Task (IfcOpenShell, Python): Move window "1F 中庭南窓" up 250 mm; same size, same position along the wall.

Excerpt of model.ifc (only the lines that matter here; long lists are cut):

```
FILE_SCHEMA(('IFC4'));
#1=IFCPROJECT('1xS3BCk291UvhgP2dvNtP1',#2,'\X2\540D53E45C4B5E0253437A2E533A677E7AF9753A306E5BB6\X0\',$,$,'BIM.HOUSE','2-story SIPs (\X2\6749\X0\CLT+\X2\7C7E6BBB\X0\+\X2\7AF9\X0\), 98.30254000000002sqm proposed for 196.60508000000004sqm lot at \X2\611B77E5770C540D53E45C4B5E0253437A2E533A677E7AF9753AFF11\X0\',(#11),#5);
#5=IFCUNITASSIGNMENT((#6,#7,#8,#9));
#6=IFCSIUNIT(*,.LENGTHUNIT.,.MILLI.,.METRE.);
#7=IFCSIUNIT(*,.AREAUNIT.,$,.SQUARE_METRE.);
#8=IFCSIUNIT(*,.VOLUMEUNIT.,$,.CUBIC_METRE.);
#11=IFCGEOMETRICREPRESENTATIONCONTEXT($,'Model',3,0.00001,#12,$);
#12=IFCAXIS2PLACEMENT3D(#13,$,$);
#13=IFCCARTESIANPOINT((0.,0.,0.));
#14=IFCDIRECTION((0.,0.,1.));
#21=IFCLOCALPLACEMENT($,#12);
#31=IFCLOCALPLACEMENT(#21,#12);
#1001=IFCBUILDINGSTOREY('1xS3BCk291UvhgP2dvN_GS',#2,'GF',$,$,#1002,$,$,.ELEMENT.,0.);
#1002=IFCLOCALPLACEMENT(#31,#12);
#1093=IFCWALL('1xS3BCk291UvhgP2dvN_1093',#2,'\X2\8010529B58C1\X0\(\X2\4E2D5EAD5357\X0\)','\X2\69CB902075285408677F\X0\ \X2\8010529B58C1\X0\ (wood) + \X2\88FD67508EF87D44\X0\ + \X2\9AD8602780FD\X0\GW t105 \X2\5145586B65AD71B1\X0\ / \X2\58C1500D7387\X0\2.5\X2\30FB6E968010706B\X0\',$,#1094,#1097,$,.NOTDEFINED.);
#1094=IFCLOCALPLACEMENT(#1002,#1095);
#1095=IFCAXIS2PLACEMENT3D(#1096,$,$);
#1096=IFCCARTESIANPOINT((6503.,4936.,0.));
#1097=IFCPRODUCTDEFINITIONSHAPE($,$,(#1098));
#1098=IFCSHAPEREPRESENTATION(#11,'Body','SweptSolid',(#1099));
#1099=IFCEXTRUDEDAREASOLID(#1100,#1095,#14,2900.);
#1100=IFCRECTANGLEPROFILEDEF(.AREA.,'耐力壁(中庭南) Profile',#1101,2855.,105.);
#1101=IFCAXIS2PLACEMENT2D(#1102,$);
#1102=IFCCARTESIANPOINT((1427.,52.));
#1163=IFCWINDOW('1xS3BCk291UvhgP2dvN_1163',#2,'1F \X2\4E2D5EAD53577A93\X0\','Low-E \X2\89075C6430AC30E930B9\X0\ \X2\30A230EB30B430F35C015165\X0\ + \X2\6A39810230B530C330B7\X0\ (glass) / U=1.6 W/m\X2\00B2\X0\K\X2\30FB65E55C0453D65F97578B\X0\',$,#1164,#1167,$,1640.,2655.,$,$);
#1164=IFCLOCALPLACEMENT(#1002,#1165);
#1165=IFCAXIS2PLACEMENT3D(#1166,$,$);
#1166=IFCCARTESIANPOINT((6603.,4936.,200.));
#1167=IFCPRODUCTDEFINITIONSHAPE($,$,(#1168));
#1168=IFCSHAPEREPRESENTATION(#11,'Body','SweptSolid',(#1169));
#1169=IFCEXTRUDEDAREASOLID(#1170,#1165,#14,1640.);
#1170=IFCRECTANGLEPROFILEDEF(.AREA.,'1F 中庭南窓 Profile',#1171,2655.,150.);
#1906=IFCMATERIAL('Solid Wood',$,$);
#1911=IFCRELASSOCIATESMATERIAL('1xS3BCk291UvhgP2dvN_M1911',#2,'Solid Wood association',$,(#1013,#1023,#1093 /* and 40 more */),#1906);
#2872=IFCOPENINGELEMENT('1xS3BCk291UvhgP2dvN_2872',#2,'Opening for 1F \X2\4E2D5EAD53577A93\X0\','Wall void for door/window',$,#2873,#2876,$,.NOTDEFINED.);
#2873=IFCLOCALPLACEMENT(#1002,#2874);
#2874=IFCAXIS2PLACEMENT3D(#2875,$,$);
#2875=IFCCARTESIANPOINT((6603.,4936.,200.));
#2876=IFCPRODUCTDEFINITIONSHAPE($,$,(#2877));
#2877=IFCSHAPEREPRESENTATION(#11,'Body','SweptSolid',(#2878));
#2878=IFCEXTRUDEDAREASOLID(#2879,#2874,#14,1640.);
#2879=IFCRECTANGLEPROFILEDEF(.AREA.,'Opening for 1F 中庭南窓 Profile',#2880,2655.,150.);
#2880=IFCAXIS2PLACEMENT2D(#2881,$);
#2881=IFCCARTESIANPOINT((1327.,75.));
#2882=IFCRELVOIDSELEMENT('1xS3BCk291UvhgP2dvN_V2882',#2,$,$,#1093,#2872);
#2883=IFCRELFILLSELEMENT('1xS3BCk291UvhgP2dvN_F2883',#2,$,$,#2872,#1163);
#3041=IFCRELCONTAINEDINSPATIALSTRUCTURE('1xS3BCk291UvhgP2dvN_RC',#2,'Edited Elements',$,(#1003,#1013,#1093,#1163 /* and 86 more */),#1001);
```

```python
import numpy as np
import ifcopenshell
import ifcopenshell.api.geometry
import ifcopenshell.util.placement
import ifcopenshell.util.unit

model = ifcopenshell.open("model.ifc")
unit_scale = ifcopenshell.util.unit.calculate_unit_scale(model)

window = model.by_guid("1xS3BCk291UvhgP2dvN_1163")
opening = window.FillsVoids[0].RelatingOpeningElement
dz = 250.0

shift = np.array([0.0, 0.0, dz])
# The window is not placed relative to its opening, so move both.
for product in (opening, window):
    matrix = ifcopenshell.util.placement.get_local_placement(product.ObjectPlacement)
    matrix[:3, 3] += shift
    ifcopenshell.api.geometry.edit_object_placement(model, product=product, matrix=matrix, is_si=False)

print(f"moved by {dz * unit_scale:+.3f} m")

model.write("model_v2.ifc")
```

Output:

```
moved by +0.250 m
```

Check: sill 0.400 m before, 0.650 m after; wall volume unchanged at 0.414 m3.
